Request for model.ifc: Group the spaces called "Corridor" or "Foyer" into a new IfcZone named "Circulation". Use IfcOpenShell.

First a look at what the model holds.

```python
import ifcopenshell

model = ifcopenshell.open("model.ifc")
print(model.schema)
seen = {}
for space in model.by_type("IfcSpace"):
    seen[space.LongName] = seen.get(space.LongName, 0) + 1
for name, count in sorted(seen.items(), key=str):
    print(count, "x", name)
print("zones:", [z.Name for z in model.by_type("IfcZone")][:20])
```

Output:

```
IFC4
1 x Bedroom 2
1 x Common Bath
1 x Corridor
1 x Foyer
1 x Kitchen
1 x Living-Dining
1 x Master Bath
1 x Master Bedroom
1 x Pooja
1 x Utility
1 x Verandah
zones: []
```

```python
import ifcopenshell
import ifcopenshell.api.group
import ifcopenshell.api.root

model = ifcopenshell.open("model.ifc")

names = {"Corridor", "Foyer"}
spaces = [s for s in model.by_type("IfcSpace") if s.LongName in names]

zone = ifcopenshell.api.root.create_entity(model, ifc_class="IfcZone", name="Circulation")
ifcopenshell.api.group.assign_group(model, products=spaces, group=zone)
print(len(spaces), "spaces in", zone.Name)

model.write("model_v2.ifc")
```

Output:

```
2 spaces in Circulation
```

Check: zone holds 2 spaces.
